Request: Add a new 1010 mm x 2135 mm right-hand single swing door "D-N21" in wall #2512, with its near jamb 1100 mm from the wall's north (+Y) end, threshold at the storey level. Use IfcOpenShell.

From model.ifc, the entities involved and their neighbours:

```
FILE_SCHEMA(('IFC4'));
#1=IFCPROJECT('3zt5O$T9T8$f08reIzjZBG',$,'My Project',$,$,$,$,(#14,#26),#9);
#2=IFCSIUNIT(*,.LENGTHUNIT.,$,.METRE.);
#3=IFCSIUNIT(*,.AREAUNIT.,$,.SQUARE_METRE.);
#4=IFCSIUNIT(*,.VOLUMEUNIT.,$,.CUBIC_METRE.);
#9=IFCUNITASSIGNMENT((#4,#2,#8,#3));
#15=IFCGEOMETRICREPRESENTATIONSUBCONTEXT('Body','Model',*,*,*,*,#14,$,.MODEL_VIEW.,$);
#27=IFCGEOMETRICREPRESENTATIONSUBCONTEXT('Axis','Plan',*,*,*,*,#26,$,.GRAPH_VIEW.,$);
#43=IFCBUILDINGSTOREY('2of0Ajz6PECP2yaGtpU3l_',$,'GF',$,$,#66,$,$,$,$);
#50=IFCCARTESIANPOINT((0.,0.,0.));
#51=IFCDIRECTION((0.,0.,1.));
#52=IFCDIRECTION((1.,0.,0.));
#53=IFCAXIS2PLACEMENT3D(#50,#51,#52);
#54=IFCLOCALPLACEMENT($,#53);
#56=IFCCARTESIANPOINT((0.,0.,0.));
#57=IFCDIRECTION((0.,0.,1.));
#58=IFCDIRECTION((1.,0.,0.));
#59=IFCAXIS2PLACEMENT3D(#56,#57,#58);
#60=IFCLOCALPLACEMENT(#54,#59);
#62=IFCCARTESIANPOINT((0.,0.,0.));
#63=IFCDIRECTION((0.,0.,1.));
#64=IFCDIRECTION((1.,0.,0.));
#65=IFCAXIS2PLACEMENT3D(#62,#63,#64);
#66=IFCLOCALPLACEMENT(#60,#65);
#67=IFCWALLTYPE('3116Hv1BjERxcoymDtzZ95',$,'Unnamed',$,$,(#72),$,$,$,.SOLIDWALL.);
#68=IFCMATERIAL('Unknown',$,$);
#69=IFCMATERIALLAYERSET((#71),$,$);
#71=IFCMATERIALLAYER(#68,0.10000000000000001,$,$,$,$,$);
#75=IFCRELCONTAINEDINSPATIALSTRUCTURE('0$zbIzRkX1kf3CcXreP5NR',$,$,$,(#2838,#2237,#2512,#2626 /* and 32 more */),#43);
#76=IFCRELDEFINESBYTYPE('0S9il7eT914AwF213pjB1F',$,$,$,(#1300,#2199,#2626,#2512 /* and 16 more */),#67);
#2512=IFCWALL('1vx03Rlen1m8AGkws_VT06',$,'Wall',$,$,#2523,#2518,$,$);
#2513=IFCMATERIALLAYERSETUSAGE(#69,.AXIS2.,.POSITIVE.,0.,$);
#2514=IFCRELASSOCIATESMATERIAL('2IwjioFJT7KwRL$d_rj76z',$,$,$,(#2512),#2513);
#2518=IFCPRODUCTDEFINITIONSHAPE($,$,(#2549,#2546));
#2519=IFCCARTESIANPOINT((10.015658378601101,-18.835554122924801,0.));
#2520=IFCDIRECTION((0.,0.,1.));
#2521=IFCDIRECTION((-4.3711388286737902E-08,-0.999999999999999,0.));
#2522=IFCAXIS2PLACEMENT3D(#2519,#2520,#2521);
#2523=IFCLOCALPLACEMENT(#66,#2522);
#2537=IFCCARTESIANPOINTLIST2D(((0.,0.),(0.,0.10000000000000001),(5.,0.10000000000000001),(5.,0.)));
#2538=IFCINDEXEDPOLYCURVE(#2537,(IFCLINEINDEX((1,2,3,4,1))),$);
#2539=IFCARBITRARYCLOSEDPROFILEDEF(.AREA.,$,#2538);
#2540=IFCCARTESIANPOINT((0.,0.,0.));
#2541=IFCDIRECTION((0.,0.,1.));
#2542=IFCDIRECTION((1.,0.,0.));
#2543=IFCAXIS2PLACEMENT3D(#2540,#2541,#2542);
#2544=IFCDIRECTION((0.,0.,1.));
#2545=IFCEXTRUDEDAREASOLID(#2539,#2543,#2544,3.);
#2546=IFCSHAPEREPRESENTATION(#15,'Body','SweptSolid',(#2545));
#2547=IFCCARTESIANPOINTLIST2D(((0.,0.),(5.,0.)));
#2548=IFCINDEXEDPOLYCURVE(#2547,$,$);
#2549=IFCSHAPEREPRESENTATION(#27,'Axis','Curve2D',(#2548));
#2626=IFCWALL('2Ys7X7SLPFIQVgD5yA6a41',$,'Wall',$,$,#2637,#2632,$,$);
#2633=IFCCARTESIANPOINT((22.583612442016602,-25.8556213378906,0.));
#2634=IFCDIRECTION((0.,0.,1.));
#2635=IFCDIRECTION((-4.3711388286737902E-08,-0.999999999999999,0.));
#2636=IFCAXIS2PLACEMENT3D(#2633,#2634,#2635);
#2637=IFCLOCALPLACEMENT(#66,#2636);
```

```python
import numpy as np
import ifcopenshell
import ifcopenshell.api.feature
import ifcopenshell.api.geometry
import ifcopenshell.api.root
import ifcopenshell.api.spatial
import ifcopenshell.geom
import ifcopenshell.util.element
import ifcopenshell.util.placement
import ifcopenshell.util.representation
import ifcopenshell.util.shape
import ifcopenshell.util.unit

model = ifcopenshell.open("model.ifc")
unit_scale = ifcopenshell.util.unit.calculate_unit_scale(model)
settings = ifcopenshell.geom.settings()


def volume(element):
    """Net volume in cubic metres, openings subtracted."""
    shape = ifcopenshell.geom.create_shape(settings, element)
    return ifcopenshell.util.shape.get_volume(shape.geometry)


wall = model.by_guid("1vx03Rlen1m8AGkws_VT06")
storey = ifcopenshell.util.element.get_container(wall, ifc_class="IfcBuildingStorey")
context = ifcopenshell.util.representation.get_context(model, "Model", "Body", "MODEL_VIEW")
before = volume(wall)

width, height, from_end, sill = 1.01, 2.135, 1.1, 0.0  # metres

# The wall runs along its own X axis, and the end named is its -X end.
wall_shape = ifcopenshell.geom.create_shape(settings, wall)
x, y, z = ifcopenshell.util.shape.get_vertices(wall_shape.geometry).T
start = x.min() + from_end
face, thickness = float(y.min()), float(y.max() - y.min())
wall_matrix = ifcopenshell.util.placement.get_local_placement(wall.ObjectPlacement)
level = ifcopenshell.util.placement.get_local_placement(storey.ObjectPlacement)[2, 3]


def in_wall(x, y):
    """Placement at x, y metres in the wall's axes, at sill height."""
    matrix = wall_matrix.copy()
    matrix[:, 3] = wall_matrix @ np.array([x / unit_scale, y / unit_scale, 0.0, 1.0])
    matrix[2, 3] = level + sill / unit_scale
    return matrix


# Opening: a box that overshoots both wall faces by 50 mm.
opening = ifcopenshell.api.root.create_entity(model, ifc_class="IfcOpeningElement", predefined_type="OPENING")
box = ifcopenshell.api.geometry.add_wall_representation(
    model, context=context, length=width, height=height, thickness=thickness + 0.1
)
ifcopenshell.api.geometry.assign_representation(model, product=opening, representation=box)
ifcopenshell.api.geometry.edit_object_placement(model, product=opening, matrix=in_wall(start, face - 0.05), is_si=False)
ifcopenshell.api.feature.add_feature(model, feature=opening, element=wall)

door = ifcopenshell.api.root.create_entity(model, ifc_class="IfcDoor", name="D-N21", predefined_type="DOOR")
door.OverallWidth, door.OverallHeight = width / unit_scale, height / unit_scale
door.OperationType = "SINGLE_SWING_RIGHT"
body = ifcopenshell.api.geometry.add_door_representation(
    model,
    context=context,
    overall_width=door.OverallWidth,
    overall_height=door.OverallHeight,
    operation_type="SINGLE_SWING_RIGHT",
    lining_properties={"LiningDepth": thickness / unit_scale, "ThresholdDepth": thickness / unit_scale},
)
ifcopenshell.api.geometry.assign_representation(model, product=door, representation=body)
ifcopenshell.api.spatial.assign_container(model, products=[door], relating_structure=storey)
ifcopenshell.api.feature.add_filling(model, opening=opening, element=door)

# The lining spans the wall, so the door starts at the wall face.
ifcopenshell.api.geometry.edit_object_placement(model, product=door, matrix=in_wall(start, face), is_si=False)

after = volume(wall)

print(f"wall volume {before:.3f} -> {after:.3f} m3")

model.write("model_edited.ifc")
```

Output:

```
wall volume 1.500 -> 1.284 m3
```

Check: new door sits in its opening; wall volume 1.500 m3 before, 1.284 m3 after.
